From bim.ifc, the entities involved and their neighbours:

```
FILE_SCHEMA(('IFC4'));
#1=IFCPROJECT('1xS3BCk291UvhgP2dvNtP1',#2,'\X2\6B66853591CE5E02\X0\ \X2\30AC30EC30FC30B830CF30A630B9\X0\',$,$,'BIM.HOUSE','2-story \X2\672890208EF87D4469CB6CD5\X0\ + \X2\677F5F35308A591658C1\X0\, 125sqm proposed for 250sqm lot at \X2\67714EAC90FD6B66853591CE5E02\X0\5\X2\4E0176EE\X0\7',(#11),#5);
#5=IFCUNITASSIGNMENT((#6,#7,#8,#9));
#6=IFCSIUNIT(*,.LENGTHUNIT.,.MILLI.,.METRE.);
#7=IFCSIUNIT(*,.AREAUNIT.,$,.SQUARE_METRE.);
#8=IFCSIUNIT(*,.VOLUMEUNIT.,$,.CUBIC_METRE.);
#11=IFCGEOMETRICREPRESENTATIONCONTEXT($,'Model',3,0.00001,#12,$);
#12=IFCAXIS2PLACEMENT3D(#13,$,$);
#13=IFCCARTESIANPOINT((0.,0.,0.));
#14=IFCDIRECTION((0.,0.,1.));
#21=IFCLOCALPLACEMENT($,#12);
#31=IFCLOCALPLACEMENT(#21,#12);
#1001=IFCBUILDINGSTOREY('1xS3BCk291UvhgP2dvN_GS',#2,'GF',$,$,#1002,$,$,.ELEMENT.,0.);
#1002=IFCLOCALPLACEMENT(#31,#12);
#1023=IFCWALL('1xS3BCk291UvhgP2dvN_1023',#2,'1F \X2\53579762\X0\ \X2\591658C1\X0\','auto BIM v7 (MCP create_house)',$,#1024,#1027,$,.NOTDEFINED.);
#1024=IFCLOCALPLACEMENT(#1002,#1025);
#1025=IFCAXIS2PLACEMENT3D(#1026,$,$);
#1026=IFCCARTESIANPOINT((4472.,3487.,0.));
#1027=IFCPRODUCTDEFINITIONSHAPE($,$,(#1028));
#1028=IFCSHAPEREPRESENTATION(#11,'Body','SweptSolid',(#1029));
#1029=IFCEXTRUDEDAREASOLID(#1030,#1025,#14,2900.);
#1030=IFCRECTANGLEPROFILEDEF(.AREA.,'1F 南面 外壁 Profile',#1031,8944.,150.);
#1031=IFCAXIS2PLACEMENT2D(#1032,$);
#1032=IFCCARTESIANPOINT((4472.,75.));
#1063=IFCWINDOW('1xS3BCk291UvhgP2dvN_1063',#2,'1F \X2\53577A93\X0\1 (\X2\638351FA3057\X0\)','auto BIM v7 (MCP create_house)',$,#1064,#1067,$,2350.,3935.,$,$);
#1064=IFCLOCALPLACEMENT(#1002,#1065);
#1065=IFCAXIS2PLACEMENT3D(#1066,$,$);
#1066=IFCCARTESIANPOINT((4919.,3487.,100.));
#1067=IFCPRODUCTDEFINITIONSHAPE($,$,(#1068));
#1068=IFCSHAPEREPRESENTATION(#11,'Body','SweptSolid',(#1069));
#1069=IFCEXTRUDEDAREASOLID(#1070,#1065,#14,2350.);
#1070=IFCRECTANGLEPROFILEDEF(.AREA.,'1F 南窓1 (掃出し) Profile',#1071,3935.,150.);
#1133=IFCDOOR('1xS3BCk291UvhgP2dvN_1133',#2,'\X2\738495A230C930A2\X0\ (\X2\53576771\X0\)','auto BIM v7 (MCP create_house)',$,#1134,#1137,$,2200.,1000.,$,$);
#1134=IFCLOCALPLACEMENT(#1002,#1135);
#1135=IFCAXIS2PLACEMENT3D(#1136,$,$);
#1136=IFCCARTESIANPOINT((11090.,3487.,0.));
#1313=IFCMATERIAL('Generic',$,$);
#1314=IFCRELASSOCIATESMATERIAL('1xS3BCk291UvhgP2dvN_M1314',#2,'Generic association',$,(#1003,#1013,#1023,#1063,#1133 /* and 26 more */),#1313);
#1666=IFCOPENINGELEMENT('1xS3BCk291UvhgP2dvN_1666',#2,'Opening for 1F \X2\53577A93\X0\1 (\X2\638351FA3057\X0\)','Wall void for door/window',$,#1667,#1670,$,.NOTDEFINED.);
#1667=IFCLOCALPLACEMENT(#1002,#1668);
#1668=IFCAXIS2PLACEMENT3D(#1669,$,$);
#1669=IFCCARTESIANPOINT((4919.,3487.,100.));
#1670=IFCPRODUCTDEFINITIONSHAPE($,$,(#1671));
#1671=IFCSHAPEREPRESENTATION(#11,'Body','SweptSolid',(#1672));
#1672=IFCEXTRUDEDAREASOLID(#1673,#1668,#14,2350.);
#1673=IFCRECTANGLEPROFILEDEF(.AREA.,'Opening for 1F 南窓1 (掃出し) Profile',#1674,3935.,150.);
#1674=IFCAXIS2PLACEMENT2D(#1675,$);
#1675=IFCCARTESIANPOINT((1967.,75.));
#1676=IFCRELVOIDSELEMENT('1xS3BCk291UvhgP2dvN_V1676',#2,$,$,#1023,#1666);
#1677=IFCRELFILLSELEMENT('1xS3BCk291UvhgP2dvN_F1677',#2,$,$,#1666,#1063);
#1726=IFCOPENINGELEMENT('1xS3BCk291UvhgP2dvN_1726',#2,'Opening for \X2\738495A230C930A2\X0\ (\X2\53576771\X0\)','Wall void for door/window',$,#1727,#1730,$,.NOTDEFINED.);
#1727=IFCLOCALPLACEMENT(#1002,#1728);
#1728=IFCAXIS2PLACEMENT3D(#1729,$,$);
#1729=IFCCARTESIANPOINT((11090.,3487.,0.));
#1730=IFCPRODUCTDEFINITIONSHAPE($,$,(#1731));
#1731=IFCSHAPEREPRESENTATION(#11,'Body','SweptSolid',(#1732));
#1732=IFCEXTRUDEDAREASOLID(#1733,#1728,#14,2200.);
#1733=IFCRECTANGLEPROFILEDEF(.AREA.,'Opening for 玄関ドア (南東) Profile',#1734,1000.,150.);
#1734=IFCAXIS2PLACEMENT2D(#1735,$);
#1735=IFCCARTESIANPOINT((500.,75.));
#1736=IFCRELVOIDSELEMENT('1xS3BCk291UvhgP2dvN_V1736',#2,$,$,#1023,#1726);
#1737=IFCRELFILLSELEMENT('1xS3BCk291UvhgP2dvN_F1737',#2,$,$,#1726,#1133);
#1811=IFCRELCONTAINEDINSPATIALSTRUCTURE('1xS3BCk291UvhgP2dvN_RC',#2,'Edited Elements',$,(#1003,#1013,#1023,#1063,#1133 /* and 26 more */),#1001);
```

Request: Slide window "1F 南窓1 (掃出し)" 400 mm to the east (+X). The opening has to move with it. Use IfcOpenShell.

```python
import ifcopenshell
import ifcopenshell.api.geometry
import ifcopenshell.util.placement
import ifcopenshell.util.unit

model = ifcopenshell.open("bim.ifc")
unit_scale = ifcopenshell.util.unit.calculate_unit_scale(model)

window = model.by_id(1063)
opening = window.FillsVoids[0].RelatingOpeningElement
wall = opening.VoidsElements[0].RelatingBuildingElement

wall_matrix = ifcopenshell.util.placement.get_local_placement(wall.ObjectPlacement)
shift = wall_matrix[:3, 0] * 0.4 / unit_scale
before = ifcopenshell.util.placement.get_local_placement(window.ObjectPlacement)[:3, 3].copy()

# The window is not placed relative to its opening, so move both.
for product in (opening, window):
    matrix = ifcopenshell.util.placement.get_local_placement(product.ObjectPlacement)
    matrix[:3, 3] += shift
    ifcopenshell.api.geometry.edit_object_placement(model, product=product, matrix=matrix, is_si=False)

after = ifcopenshell.util.placement.get_local_placement(window.ObjectPlacement)[:3, 3]
print("window moved by", (after - before).round(3) + 0.0)

model.write("bim-out.ifc")
```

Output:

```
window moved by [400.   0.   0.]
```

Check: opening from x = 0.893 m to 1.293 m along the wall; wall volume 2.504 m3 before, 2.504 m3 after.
